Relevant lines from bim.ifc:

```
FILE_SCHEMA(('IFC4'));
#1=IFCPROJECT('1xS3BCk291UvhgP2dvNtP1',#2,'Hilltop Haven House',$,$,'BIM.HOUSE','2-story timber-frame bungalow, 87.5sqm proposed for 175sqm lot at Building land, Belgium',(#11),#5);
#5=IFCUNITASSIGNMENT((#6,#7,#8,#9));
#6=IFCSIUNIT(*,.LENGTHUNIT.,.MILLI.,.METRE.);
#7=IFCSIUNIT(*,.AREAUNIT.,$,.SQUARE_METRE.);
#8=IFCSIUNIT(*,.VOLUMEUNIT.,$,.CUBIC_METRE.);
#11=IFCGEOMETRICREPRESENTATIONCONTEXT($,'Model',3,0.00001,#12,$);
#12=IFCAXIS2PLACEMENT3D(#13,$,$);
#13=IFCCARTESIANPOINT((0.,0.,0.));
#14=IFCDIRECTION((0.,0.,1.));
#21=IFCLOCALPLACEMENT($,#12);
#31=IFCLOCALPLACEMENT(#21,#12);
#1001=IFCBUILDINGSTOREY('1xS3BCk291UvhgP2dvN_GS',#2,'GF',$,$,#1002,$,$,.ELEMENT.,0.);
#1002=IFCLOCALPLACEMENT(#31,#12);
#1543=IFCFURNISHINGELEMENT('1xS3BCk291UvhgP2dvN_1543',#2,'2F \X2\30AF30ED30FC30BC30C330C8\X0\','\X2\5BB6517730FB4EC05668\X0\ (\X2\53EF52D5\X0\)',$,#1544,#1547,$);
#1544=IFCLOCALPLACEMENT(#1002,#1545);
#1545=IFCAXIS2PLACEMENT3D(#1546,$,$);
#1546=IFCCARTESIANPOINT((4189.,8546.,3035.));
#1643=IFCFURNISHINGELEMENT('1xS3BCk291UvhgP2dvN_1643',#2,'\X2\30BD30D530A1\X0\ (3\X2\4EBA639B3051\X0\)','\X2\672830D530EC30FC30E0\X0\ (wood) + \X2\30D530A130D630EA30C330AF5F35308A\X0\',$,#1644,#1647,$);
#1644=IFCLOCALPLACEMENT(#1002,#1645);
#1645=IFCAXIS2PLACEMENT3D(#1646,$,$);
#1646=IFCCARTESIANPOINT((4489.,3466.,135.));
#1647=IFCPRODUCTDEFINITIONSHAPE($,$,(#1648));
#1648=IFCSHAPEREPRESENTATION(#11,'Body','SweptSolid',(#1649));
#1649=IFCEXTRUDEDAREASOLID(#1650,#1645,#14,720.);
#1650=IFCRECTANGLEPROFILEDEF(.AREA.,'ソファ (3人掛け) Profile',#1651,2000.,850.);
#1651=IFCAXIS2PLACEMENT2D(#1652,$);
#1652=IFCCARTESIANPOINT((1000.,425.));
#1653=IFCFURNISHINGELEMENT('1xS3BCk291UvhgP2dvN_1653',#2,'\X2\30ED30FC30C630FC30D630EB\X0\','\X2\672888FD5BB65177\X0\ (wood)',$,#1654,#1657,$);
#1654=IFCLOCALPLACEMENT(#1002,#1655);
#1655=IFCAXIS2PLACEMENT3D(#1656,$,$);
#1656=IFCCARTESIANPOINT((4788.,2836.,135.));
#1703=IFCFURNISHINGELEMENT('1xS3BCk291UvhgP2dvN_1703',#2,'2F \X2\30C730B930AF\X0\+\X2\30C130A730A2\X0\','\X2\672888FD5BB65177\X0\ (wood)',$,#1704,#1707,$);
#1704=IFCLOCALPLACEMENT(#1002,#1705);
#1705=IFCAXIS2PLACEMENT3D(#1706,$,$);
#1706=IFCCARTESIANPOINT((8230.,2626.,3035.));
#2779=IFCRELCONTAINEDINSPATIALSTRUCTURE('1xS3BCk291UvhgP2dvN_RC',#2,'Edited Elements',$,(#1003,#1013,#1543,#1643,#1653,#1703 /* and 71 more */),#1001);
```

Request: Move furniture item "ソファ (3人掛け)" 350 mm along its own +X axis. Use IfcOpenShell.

```python
import ifcopenshell
import ifcopenshell.api.geometry
import ifcopenshell.util.placement
import ifcopenshell.util.unit

model = ifcopenshell.open("bim.ifc")
unit_scale = ifcopenshell.util.unit.calculate_unit_scale(model)

item = model.by_id(1643)
matrix = ifcopenshell.util.placement.get_local_placement(item.ObjectPlacement)
matrix[:3, 3] += matrix[:3, 0] * 0.35 / unit_scale
ifcopenshell.api.geometry.edit_object_placement(model, product=item, matrix=matrix, is_si=False)

print(ifcopenshell.util.placement.get_local_placement(item.ObjectPlacement).round(3) + 0.0)

model.write("bim_v2.ifc")
```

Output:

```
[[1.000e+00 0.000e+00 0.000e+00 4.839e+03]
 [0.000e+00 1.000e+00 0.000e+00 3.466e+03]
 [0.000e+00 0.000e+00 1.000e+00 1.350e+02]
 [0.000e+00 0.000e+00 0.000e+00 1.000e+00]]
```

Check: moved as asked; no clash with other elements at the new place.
